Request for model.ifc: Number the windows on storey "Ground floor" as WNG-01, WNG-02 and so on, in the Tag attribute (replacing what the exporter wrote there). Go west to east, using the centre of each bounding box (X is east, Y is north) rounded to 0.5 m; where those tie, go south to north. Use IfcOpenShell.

First a look at what the model holds.

```python
import ifcopenshell
import ifcopenshell.util.element
import ifcopenshell.util.placement

model = ifcopenshell.open("model.ifc")
print(model.schema)
storey = next(s for s in model.by_type("IfcBuildingStorey") if s.Name == "Ground floor")
windows = [e for e in ifcopenshell.util.element.get_decomposition(storey) if e.is_a("IfcWindow")]
for e in sorted(windows, key=lambda e: e.id()):
    origin = ifcopenshell.util.placement.get_local_placement(e.ObjectPlacement)[:3, 3]
    print(e.id(), e.Tag, e.Name, origin.round(2) + 0.0, sep=" | ")
```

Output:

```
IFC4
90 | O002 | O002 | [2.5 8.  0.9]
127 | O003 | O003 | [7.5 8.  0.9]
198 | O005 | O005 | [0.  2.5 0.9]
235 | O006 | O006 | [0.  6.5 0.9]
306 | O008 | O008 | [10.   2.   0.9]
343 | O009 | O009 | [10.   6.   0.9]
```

```python
import ifcopenshell
import ifcopenshell.geom
import ifcopenshell.util.element
import ifcopenshell.util.shape

model = ifcopenshell.open("model.ifc")
settings = ifcopenshell.geom.settings()
settings.set("use-world-coords", True)


def centre(element):
    shape = ifcopenshell.geom.create_shape(settings, element)
    return ifcopenshell.util.shape.get_bbox_centroid(shape.geometry)


storey = next(s for s in model.by_type("IfcBuildingStorey") if s.Name == "Ground floor")
windows = [e for e in ifcopenshell.util.element.get_decomposition(storey) if e.is_a("IfcWindow")]

# Insertion points can sit at a corner or the storey origin, so sort by the geometry (in metres).
centres = {e: centre(e) for e in windows}
windows.sort(key=lambda e: (round(centres[e][0] / 0.5), centres[e][1]))

for i, e in enumerate(windows, start=1):
    number = f"WNG-{i:02d}"
    e.Tag = number
    print(e.id(), number)

model.write("model_edited.ifc")
```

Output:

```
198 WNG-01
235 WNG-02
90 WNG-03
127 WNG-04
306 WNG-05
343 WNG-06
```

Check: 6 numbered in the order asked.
